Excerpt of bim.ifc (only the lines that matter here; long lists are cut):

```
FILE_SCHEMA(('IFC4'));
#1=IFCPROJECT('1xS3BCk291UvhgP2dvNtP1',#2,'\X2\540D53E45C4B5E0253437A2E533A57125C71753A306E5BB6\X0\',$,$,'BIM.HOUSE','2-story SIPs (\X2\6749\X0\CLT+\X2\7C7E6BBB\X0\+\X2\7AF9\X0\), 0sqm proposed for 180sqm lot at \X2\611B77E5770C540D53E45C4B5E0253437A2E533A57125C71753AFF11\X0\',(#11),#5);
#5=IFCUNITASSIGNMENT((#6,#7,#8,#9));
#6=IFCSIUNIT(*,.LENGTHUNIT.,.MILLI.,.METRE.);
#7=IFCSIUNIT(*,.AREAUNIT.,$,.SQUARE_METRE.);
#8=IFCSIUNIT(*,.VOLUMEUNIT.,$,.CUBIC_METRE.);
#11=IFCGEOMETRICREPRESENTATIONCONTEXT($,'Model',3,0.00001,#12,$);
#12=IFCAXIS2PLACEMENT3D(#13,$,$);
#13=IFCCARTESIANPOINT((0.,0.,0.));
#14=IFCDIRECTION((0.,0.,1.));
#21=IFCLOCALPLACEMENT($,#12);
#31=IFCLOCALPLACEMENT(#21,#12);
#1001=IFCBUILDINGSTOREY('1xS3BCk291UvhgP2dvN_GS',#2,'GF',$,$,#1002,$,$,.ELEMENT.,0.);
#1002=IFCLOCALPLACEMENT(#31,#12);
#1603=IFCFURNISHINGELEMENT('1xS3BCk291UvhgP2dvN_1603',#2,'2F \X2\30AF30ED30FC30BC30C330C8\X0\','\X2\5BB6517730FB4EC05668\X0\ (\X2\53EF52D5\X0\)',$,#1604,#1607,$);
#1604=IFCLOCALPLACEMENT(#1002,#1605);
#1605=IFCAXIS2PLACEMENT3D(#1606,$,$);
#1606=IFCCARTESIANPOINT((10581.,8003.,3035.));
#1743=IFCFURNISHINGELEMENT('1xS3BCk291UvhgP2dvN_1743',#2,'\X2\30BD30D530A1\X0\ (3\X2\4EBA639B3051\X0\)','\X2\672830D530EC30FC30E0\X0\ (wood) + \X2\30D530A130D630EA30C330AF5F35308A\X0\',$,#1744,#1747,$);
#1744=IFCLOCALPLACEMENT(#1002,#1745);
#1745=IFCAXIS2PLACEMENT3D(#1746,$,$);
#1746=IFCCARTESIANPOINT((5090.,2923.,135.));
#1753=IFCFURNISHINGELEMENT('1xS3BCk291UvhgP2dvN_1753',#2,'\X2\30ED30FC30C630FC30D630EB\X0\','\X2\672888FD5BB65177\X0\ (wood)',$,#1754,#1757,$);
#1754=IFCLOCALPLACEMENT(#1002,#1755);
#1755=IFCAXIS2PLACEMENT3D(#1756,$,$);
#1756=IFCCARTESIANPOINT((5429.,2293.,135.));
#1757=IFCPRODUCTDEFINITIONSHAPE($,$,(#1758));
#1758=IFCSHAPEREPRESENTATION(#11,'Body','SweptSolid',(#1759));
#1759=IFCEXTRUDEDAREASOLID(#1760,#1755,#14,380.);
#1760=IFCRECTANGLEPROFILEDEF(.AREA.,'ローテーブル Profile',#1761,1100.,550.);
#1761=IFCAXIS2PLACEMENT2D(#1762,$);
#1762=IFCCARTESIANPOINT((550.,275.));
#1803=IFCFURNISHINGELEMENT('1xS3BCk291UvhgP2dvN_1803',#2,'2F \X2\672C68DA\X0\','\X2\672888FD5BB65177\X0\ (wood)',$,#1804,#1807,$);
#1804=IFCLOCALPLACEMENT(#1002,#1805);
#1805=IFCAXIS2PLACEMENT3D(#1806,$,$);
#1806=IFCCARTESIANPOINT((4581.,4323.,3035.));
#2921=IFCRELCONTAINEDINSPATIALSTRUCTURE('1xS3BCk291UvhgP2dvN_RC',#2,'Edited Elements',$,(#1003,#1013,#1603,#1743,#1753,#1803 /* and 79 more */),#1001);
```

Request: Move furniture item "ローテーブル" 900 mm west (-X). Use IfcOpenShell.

```python
import ifcopenshell
import ifcopenshell.api.geometry
import ifcopenshell.util.placement
import ifcopenshell.util.unit

model = ifcopenshell.open("bim.ifc")
unit_scale = ifcopenshell.util.unit.calculate_unit_scale(model)

item = model.by_guid("1xS3BCk291UvhgP2dvN_1753")
matrix = ifcopenshell.util.placement.get_local_placement(item.ObjectPlacement)
matrix[0, 3] -= 0.9 / unit_scale
ifcopenshell.api.geometry.edit_object_placement(model, product=item, matrix=matrix, is_si=False)

print(ifcopenshell.util.placement.get_local_placement(item.ObjectPlacement).round(3) + 0.0)

model.write("bim_updated.ifc")
```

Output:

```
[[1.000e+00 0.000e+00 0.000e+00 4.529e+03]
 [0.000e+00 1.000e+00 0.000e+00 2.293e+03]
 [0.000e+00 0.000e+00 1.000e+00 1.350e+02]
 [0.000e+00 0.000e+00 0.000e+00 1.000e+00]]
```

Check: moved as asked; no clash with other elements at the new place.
